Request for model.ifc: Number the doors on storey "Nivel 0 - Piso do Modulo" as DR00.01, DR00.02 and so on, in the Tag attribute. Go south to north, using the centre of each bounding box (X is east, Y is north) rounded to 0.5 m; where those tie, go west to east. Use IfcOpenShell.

First a look at what the model holds.

```python
import ifcopenshell
import ifcopenshell.util.element
import ifcopenshell.util.placement

model = ifcopenshell.open("model.ifc")
print(model.schema)
storey = next(s for s in model.by_type("IfcBuildingStorey") if s.Name == "Nivel 0 - Piso do Modulo")
doors = [e for e in ifcopenshell.util.element.get_decomposition(storey) if e.is_a("IfcDoor")]
for e in sorted(doors, key=lambda e: e.id()):
    origin = ifcopenshell.util.placement.get_local_placement(e.ObjectPlacement)[:3, 3]
    print(e.id(), e.Tag, e.Name, origin.round(2) + 0.0, sep=" | ")
```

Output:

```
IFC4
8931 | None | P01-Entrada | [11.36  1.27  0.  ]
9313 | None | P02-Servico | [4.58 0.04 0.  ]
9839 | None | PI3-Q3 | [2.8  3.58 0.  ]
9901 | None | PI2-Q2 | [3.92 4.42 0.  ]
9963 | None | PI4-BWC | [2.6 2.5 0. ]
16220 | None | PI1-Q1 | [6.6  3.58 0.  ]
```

```python
import ifcopenshell
import ifcopenshell.geom
import ifcopenshell.util.element
import ifcopenshell.util.shape

model = ifcopenshell.open("model.ifc")
settings = ifcopenshell.geom.settings()
settings.set("use-world-coords", True)


def centre(element):
    shape = ifcopenshell.geom.create_shape(settings, element)
    return ifcopenshell.util.shape.get_bbox_centroid(shape.geometry)


storey = next(s for s in model.by_type("IfcBuildingStorey") if s.Name == "Nivel 0 - Piso do Modulo")
doors = [e for e in ifcopenshell.util.element.get_decomposition(storey) if e.is_a("IfcDoor")]

# Insertion points can sit at a corner or the storey origin, so sort by the geometry (in metres).
centres = {e: centre(e) for e in doors}
doors.sort(key=lambda e: (round(centres[e][1] / 0.5), centres[e][0]))

for i, e in enumerate(doors, start=1):
    number = f"DR00.{i:02d}"
    e.Tag = number
    print(e.id(), number)

model.write("model_v2.ifc")
```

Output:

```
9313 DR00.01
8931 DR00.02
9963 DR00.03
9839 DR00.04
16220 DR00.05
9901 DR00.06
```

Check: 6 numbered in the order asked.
